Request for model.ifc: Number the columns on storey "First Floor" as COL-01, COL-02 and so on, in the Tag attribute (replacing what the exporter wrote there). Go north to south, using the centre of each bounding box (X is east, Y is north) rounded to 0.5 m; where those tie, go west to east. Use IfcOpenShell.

First a look at what the model holds.

```python
import ifcopenshell
import ifcopenshell.util.element
import ifcopenshell.util.placement

model = ifcopenshell.open("model.ifc")
print(model.schema)
storey = next(s for s in model.by_type("IfcBuildingStorey") if s.Name == "First Floor")
columns = [e for e in ifcopenshell.util.element.get_decomposition(storey) if e.is_a("IfcColumn")]
for e in sorted(columns, key=lambda e: e.id()):
    origin = ifcopenshell.util.placement.get_local_placement(e.ObjectPlacement)[:3, 3]
    print(e.id(), e.Tag, e.Name, origin.round(2) + 0.0, sep=" | ")
```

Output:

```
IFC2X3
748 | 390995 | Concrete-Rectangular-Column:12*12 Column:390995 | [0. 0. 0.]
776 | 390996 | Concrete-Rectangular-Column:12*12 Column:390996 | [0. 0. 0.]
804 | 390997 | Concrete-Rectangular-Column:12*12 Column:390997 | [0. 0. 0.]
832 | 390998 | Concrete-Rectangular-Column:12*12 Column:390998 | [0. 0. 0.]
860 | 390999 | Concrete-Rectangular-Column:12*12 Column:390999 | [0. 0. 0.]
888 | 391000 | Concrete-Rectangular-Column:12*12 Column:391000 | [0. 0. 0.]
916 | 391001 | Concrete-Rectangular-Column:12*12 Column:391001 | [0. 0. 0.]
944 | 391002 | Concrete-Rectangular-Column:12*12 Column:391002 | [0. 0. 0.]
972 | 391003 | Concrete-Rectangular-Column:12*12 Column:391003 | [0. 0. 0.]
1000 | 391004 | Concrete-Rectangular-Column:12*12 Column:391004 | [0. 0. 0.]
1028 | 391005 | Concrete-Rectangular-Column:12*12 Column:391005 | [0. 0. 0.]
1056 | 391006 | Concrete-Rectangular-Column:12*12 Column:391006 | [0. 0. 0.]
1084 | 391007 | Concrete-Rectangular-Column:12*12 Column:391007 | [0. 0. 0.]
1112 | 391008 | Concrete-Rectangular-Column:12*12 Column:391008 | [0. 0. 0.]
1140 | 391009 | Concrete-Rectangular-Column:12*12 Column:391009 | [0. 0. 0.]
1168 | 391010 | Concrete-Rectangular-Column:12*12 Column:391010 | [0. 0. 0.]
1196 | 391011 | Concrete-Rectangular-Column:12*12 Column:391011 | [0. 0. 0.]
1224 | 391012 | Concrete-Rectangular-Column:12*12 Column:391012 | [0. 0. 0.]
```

```python
import ifcopenshell
import ifcopenshell.geom
import ifcopenshell.util.element
import ifcopenshell.util.shape

model = ifcopenshell.open("model.ifc")
settings = ifcopenshell.geom.settings()
settings.set("use-world-coords", True)


def centre(element):
    shape = ifcopenshell.geom.create_shape(settings, element)
    return ifcopenshell.util.shape.get_bbox_centroid(shape.geometry)


storey = next(s for s in model.by_type("IfcBuildingStorey") if s.Name == "First Floor")
columns = [e for e in ifcopenshell.util.element.get_decomposition(storey) if e.is_a("IfcColumn")]

# Insertion points can sit at a corner or the storey origin, so sort by the geometry (in metres).
centres = {e: centre(e) for e in columns}
columns.sort(key=lambda e: (-round(centres[e][1] / 0.5), centres[e][0]))

for i, e in enumerate(columns, start=1):
    number = f"COL-{i:02d}"
    e.Tag = number
    print(e.id(), number)

model.write("model-out.ifc")
```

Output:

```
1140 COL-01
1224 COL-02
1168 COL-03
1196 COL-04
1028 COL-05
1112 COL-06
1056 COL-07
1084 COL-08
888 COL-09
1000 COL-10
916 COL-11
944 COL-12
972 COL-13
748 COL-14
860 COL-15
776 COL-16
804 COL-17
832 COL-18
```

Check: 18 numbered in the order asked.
